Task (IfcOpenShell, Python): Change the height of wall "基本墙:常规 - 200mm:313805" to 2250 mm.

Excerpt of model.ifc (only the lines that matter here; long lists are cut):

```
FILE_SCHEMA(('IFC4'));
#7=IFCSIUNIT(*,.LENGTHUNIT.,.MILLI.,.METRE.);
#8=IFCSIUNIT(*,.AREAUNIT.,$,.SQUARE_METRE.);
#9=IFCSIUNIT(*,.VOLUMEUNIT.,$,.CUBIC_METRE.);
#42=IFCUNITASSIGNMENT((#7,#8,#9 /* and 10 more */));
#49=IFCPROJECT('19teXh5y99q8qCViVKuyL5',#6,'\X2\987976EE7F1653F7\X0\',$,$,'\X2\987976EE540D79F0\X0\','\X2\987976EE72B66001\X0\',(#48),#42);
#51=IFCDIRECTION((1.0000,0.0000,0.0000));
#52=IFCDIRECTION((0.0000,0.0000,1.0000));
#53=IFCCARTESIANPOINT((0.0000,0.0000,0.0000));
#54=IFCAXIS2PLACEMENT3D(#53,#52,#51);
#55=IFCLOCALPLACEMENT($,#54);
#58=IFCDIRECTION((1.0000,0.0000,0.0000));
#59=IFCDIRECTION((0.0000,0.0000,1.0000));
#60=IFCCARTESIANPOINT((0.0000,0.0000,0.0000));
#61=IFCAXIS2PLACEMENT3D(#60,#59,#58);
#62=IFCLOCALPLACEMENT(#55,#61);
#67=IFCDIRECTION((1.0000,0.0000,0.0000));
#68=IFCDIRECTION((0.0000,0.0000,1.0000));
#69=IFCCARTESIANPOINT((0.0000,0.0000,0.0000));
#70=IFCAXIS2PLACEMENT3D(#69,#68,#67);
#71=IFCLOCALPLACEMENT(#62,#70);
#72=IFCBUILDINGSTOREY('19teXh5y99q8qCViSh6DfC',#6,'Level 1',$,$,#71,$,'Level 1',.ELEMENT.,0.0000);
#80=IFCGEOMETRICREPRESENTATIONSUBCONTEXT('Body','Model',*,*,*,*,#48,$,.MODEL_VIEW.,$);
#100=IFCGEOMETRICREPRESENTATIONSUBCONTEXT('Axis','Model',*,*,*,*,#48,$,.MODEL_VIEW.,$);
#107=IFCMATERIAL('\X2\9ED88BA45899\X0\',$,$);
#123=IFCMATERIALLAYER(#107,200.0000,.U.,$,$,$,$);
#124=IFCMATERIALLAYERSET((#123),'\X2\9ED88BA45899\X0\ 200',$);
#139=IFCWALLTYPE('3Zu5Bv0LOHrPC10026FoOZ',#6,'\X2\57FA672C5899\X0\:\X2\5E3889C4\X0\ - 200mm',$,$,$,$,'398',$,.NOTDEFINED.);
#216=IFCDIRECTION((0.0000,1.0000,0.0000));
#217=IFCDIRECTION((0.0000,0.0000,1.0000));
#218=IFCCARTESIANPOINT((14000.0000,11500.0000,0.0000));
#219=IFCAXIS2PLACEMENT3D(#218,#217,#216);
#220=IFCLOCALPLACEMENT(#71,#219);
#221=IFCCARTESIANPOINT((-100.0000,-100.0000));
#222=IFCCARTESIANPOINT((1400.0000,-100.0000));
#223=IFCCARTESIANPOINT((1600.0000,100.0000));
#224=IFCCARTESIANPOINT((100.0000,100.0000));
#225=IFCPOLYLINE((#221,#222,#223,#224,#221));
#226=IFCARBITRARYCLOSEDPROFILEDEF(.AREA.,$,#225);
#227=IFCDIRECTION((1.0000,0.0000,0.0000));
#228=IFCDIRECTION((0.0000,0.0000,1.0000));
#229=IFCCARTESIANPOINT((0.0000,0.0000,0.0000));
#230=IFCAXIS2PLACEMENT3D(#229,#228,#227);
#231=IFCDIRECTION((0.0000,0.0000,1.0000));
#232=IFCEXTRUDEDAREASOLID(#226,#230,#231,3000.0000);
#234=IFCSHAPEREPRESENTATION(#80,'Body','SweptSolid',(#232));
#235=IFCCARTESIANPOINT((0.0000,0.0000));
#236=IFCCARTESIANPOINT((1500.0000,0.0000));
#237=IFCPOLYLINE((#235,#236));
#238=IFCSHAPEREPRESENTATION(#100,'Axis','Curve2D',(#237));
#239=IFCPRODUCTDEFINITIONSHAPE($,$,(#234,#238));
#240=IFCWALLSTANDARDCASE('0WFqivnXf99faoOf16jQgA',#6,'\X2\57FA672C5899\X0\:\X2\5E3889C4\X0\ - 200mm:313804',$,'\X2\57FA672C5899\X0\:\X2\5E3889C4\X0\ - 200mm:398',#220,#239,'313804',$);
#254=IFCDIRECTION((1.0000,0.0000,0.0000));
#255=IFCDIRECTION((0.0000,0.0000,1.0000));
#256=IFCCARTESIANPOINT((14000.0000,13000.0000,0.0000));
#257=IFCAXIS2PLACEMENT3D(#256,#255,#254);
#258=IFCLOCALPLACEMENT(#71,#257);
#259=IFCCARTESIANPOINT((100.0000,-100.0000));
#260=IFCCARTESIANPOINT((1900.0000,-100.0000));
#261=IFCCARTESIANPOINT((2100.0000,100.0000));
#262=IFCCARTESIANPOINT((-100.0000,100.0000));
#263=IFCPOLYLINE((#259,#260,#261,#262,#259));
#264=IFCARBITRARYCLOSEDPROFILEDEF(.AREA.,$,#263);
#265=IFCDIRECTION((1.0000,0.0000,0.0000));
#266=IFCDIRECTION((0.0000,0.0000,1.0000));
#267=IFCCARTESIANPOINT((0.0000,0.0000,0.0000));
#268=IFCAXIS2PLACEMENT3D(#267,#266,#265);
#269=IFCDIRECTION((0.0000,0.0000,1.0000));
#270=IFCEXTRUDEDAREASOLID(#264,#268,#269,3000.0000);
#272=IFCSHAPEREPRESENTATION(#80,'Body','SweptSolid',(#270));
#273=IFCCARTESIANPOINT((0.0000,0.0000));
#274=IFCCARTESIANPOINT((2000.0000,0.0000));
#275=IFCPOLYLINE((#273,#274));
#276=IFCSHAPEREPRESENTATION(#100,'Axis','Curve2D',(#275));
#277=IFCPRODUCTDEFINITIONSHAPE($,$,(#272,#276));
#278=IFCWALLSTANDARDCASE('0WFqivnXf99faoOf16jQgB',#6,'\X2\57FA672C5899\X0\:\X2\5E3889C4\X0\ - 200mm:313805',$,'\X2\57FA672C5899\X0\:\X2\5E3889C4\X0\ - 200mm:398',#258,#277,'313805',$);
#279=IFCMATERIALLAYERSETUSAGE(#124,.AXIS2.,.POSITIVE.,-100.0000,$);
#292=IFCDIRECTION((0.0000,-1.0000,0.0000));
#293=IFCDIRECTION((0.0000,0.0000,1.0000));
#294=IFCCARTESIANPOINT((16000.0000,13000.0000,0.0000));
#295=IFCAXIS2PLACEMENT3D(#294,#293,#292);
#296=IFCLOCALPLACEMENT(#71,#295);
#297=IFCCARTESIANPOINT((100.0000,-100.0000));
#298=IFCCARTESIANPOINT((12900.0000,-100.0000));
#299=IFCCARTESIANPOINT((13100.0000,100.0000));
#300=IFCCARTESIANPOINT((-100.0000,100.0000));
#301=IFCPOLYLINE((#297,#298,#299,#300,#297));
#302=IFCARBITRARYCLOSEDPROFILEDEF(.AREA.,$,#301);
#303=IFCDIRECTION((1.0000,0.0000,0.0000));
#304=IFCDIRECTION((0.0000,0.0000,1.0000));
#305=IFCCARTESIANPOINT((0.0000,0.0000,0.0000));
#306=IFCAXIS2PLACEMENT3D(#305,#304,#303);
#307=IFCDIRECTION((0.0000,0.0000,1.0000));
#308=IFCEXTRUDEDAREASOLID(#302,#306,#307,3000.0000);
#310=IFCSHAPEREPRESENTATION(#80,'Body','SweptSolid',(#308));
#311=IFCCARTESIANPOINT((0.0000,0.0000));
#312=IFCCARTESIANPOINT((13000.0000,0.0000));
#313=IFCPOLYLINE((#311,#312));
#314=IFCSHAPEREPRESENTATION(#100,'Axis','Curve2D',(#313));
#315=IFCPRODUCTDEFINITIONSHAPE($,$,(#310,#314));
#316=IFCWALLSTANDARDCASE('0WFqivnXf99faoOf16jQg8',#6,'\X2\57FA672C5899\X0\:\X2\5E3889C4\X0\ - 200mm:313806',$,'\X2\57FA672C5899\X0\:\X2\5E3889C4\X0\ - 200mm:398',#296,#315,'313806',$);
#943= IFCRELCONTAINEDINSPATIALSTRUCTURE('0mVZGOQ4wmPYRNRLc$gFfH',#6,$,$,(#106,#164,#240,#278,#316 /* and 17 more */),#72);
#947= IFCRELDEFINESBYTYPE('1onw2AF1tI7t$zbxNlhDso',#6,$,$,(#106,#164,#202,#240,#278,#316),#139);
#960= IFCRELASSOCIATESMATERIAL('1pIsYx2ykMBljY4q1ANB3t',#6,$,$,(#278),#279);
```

```python
import ifcopenshell
import ifcopenshell.geom
import ifcopenshell.util.representation
import ifcopenshell.util.shape
import ifcopenshell.util.unit

model = ifcopenshell.open("model.ifc")
unit_scale = ifcopenshell.util.unit.calculate_unit_scale(model)
settings = ifcopenshell.geom.settings()


def volume(element):
    """Net volume in cubic metres, openings subtracted."""
    shape = ifcopenshell.geom.create_shape(settings, element)
    return ifcopenshell.util.shape.get_volume(shape.geometry)


wall = model.by_id(278)
before = volume(wall)

body = ifcopenshell.util.representation.get_representation(wall, "Model", "Body")
solid = body.Items[0]
old_height = solid.Depth
solid.Depth = 2.25 / unit_scale
after = volume(wall)

print(f"height {old_height:g} -> {solid.Depth:g}, volume {before:.3f} -> {after:.3f} m3")

model.write("model_v2.ifc")
```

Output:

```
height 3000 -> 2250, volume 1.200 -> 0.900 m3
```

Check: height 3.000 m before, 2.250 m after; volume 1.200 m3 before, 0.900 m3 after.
